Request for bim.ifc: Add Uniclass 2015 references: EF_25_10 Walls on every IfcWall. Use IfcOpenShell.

First a look at what the model holds.

```python
import ifcopenshell

model = ifcopenshell.open("bim.ifc")
print(model.schema)
print("classifications:", [c.Name for c in model.by_type("IfcClassification")])
for ifc_class in ("IfcDoor", "IfcRoof", "IfcStair", "IfcWall", "IfcWindow"):
    print(ifc_class, len(model.by_type(ifc_class)))
```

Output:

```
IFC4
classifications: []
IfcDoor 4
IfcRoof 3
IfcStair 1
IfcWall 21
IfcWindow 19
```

```python
import ifcopenshell
import ifcopenshell.api.classification

model = ifcopenshell.open("bim.ifc")

system = ifcopenshell.api.classification.add_classification(model, classification="Uniclass 2015")

codes = {
    "IfcWall": ("EF_25_10", "Walls"),
}
for ifc_class, (code, name) in codes.items():
    products = model.by_type(ifc_class)
    ifcopenshell.api.classification.add_reference(
        model, products=products, classification=system, identification=code, name=name
    )
    print(code, len(products))

model.write("bim_v2.ifc")
```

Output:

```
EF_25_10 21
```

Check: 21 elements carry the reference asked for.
